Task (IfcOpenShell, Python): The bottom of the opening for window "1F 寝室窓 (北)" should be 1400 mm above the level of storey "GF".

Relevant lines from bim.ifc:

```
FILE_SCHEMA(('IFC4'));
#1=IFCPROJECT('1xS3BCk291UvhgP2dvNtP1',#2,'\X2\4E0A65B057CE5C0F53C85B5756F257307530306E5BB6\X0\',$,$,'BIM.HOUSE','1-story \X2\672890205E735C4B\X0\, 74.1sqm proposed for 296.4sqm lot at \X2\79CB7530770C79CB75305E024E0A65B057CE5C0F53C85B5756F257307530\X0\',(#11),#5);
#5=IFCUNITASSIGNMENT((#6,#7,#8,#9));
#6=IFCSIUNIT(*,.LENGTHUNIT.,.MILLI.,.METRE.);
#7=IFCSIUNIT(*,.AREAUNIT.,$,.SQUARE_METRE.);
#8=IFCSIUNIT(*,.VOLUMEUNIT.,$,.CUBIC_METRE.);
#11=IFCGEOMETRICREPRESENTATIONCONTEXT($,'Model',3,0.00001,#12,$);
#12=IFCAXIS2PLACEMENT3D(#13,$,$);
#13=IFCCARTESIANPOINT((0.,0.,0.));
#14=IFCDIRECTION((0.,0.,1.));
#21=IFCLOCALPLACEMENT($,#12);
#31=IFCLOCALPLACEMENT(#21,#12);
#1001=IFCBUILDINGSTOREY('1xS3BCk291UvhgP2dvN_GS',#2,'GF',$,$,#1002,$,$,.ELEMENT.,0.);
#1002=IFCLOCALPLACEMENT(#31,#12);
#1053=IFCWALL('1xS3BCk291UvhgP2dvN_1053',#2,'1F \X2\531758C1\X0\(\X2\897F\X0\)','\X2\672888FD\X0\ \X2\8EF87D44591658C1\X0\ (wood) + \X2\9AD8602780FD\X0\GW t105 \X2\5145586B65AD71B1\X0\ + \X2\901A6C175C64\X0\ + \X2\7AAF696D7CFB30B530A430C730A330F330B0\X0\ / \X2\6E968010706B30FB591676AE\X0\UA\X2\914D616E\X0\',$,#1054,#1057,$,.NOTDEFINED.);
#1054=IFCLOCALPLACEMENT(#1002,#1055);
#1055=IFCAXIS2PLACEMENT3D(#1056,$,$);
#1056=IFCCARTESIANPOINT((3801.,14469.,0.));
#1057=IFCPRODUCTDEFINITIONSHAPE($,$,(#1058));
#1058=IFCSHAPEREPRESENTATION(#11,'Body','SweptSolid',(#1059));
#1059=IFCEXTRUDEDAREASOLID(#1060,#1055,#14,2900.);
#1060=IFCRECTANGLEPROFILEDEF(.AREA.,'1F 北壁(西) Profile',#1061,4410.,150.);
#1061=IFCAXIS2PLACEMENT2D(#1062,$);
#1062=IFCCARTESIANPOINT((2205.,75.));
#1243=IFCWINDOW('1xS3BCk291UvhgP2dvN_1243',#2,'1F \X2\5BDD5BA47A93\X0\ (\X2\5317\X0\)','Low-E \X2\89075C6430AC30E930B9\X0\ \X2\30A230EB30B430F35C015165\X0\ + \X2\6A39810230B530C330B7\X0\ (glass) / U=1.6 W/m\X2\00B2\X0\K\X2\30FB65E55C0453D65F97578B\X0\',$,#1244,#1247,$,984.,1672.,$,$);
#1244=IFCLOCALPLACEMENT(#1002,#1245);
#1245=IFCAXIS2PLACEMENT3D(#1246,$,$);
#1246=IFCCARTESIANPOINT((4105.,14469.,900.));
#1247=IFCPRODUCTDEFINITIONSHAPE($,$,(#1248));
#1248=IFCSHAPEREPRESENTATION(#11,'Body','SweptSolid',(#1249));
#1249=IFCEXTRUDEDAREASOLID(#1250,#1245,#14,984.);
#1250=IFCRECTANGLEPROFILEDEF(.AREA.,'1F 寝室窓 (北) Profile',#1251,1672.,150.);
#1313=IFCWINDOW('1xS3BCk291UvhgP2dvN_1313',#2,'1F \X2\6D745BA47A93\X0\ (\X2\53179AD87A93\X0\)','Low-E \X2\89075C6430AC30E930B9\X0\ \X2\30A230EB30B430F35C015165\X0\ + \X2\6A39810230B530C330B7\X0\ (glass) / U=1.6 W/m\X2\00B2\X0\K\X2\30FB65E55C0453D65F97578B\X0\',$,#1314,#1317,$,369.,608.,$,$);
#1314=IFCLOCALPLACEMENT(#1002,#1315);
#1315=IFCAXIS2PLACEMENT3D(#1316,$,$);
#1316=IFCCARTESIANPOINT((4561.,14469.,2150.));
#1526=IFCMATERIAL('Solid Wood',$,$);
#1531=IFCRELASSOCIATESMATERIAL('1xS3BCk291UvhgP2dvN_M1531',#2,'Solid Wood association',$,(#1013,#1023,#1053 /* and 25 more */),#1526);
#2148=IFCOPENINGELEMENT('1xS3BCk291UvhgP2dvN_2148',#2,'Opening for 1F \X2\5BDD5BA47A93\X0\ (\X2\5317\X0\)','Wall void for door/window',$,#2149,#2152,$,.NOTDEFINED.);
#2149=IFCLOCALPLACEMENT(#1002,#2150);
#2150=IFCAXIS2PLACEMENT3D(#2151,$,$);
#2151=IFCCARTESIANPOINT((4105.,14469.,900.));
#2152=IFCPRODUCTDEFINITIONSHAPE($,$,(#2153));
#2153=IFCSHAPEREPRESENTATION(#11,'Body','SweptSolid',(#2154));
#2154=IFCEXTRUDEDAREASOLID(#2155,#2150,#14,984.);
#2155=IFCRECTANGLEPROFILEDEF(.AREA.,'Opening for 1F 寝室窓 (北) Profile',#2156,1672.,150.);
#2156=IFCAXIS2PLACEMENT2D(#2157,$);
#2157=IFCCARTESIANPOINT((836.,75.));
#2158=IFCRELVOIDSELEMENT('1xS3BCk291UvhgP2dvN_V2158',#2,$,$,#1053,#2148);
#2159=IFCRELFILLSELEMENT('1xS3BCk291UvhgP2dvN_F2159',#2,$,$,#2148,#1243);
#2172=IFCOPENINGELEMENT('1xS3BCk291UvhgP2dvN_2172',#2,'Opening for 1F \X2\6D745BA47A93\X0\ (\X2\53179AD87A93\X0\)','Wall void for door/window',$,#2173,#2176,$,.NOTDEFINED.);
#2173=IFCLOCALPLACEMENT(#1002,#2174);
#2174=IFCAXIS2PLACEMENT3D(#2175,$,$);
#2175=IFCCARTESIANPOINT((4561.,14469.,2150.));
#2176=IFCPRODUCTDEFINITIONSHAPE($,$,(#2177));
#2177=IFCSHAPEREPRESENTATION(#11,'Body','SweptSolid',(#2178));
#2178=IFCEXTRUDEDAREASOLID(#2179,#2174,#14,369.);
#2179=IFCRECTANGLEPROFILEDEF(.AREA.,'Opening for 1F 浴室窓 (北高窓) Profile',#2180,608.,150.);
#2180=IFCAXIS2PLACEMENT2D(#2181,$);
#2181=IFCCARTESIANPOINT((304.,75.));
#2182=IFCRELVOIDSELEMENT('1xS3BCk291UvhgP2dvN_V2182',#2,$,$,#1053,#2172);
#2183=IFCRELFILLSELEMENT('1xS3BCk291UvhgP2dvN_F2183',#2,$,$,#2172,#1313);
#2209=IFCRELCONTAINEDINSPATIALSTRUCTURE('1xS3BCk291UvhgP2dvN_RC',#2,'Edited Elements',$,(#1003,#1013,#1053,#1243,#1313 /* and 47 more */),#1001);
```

```python
import numpy as np
import ifcopenshell
import ifcopenshell.api.geometry
import ifcopenshell.geom
import ifcopenshell.util.element
import ifcopenshell.util.placement
import ifcopenshell.util.shape
import ifcopenshell.util.unit

model = ifcopenshell.open("bim.ifc")
unit_scale = ifcopenshell.util.unit.calculate_unit_scale(model)

window = model.by_guid("1xS3BCk291UvhgP2dvN_1243")
opening = window.FillsVoids[0].RelatingOpeningElement
storey = ifcopenshell.util.element.get_container(window, ifc_class="IfcBuildingStorey")
level = ifcopenshell.util.placement.get_local_placement(storey.ObjectPlacement)[2, 3]

# The opening's origin need not be at the sill, so measure its lowest point.
shape = ifcopenshell.geom.create_shape(ifcopenshell.geom.settings(), opening)
bottom = ifcopenshell.util.shape.get_shape_bottom_elevation(shape, shape.geometry) / unit_scale
dz = level + 1400.0 - bottom

shift = np.array([0.0, 0.0, dz])
# The window is not placed relative to its opening, so move both.
for product in (opening, window):
    matrix = ifcopenshell.util.placement.get_local_placement(product.ObjectPlacement)
    matrix[:3, 3] += shift
    ifcopenshell.api.geometry.edit_object_placement(model, product=product, matrix=matrix, is_si=False)

print(f"moved by {dz * unit_scale:+.3f} m")

model.write("bim_edited.ifc")
```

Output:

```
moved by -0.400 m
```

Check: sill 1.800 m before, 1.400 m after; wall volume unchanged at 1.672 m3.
